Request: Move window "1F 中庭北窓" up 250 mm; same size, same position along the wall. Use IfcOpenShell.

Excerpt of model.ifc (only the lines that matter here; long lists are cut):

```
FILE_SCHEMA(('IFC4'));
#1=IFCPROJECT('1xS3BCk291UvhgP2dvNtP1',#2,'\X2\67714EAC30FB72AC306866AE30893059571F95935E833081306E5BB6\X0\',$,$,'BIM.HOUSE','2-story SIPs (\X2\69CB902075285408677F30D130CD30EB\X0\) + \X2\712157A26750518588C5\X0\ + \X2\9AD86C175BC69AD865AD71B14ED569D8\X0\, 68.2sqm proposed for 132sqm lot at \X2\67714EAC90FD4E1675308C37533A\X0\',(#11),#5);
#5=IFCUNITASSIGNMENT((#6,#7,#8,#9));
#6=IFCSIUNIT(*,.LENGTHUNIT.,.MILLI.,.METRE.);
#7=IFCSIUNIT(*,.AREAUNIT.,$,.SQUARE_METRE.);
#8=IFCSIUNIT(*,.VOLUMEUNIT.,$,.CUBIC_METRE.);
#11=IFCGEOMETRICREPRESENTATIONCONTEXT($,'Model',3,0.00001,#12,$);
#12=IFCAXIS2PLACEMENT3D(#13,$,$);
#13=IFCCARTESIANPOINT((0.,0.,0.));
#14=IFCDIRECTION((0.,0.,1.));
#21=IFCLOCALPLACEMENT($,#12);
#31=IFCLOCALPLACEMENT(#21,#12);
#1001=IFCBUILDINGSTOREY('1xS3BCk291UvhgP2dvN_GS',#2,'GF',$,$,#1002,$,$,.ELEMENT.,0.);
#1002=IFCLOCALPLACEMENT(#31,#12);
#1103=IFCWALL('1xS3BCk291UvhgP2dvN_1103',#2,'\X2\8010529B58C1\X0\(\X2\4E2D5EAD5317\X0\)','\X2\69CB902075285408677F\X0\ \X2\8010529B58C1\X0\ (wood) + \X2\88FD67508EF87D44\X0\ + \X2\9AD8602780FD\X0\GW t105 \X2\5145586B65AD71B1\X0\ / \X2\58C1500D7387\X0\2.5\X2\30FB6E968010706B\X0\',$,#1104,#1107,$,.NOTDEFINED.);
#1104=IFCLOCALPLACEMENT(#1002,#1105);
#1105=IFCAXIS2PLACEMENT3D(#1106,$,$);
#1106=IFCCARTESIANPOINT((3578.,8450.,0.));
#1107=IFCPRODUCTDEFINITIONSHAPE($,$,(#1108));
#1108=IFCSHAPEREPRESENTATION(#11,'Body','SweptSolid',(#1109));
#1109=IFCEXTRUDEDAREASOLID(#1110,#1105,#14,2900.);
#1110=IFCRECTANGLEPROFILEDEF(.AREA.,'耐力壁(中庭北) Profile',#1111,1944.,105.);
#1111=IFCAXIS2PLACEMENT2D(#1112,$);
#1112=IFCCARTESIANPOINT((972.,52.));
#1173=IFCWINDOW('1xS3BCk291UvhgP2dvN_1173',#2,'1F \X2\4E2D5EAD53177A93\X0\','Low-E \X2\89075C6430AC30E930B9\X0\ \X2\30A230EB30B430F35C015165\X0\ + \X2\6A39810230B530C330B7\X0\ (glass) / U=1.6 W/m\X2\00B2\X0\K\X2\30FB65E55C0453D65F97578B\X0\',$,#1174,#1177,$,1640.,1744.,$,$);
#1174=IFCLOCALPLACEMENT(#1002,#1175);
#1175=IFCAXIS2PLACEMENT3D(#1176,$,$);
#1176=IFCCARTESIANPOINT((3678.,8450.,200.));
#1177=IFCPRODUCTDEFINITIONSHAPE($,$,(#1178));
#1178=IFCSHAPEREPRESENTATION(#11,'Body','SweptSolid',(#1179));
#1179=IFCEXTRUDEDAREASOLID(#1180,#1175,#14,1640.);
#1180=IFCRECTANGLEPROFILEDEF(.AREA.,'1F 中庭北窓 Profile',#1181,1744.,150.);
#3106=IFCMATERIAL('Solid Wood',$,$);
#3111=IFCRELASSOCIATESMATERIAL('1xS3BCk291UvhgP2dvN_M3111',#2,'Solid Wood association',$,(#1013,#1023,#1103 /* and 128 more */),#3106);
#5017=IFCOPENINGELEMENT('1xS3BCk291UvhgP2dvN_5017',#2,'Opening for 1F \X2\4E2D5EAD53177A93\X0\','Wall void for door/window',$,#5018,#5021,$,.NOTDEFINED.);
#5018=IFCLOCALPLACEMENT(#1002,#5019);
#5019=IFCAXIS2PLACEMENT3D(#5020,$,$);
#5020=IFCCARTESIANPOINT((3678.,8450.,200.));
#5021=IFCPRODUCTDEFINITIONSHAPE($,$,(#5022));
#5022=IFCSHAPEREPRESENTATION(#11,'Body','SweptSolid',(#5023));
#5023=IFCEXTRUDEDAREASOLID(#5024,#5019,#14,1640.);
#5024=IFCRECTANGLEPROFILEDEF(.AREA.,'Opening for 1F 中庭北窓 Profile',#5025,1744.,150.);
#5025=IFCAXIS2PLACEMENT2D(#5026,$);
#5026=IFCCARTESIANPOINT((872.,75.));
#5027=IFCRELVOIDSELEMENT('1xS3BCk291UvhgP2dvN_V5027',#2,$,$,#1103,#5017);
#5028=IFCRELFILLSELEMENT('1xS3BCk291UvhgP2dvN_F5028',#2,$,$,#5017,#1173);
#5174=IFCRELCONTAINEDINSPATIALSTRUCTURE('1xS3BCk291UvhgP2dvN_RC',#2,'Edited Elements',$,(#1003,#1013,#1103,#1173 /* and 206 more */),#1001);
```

```python
import numpy as np
import ifcopenshell
import ifcopenshell.api.geometry
import ifcopenshell.util.placement
import ifcopenshell.util.unit

model = ifcopenshell.open("model.ifc")
unit_scale = ifcopenshell.util.unit.calculate_unit_scale(model)

window = model.by_guid("1xS3BCk291UvhgP2dvN_1173")
opening = window.FillsVoids[0].RelatingOpeningElement
dz = 0.25 / unit_scale

shift = np.array([0.0, 0.0, dz])
# The window is not placed relative to its opening, so move both.
for product in (opening, window):
    matrix = ifcopenshell.util.placement.get_local_placement(product.ObjectPlacement)
    matrix[:3, 3] += shift
    ifcopenshell.api.geometry.edit_object_placement(model, product=product, matrix=matrix, is_si=False)

print(f"moved by {dz * unit_scale:+.3f} m")

model.write("model-out.ifc")
```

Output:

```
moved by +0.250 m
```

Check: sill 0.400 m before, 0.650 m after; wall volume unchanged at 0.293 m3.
